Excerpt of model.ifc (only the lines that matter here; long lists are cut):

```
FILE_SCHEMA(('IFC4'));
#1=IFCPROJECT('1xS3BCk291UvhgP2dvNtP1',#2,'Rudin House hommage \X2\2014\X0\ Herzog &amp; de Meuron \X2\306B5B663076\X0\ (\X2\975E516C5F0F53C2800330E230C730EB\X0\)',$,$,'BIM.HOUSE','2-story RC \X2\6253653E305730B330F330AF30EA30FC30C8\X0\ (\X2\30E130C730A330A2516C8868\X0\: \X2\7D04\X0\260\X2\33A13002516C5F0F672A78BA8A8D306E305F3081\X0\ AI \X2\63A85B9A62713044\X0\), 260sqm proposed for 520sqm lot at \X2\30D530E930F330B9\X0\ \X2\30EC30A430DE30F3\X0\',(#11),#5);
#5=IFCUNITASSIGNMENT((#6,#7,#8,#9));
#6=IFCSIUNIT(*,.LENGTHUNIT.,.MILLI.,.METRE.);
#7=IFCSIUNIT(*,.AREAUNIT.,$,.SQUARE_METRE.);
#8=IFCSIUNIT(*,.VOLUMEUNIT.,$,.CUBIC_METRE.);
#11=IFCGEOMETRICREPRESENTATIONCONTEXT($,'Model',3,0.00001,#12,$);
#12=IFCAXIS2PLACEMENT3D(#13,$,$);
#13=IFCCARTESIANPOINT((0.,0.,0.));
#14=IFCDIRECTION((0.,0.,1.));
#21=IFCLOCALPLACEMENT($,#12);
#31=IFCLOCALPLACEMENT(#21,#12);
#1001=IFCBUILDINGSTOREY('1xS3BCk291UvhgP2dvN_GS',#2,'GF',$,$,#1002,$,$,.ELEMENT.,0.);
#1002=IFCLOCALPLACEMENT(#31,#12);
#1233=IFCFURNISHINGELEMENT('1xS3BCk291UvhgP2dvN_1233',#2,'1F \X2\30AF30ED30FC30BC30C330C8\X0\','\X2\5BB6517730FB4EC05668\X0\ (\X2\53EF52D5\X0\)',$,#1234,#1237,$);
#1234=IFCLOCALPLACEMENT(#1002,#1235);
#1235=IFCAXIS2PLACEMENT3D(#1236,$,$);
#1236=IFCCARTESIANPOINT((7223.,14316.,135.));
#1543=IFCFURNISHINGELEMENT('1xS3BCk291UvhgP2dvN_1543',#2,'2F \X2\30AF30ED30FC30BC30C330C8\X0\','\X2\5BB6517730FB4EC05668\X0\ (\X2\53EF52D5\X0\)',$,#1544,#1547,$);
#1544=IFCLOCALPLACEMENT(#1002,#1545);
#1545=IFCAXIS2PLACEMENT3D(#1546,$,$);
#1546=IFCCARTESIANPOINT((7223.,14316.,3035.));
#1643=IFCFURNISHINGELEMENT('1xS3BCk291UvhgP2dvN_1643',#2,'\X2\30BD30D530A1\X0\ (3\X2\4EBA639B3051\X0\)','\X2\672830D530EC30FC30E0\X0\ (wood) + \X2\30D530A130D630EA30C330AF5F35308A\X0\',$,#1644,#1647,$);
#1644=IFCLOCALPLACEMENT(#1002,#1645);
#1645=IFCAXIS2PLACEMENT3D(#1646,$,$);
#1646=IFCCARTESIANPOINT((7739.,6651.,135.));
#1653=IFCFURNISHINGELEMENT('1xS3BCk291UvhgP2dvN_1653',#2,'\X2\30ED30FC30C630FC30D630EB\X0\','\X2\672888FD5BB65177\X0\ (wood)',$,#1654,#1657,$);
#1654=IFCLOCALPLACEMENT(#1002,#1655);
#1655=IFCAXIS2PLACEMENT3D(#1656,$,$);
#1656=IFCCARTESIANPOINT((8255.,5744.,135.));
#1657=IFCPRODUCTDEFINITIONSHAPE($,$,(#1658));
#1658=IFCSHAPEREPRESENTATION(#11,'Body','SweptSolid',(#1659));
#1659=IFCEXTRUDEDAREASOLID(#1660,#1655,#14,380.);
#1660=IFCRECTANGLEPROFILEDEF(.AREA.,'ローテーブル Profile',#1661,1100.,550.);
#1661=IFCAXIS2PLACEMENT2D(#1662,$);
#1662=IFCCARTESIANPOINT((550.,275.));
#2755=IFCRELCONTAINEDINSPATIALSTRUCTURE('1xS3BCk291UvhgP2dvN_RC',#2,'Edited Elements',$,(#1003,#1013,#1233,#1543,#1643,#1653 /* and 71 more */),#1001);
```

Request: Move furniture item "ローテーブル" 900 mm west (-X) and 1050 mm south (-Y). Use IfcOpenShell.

```python
import ifcopenshell
import ifcopenshell.api.geometry
import ifcopenshell.util.placement
import ifcopenshell.util.unit

model = ifcopenshell.open("model.ifc")
unit_scale = ifcopenshell.util.unit.calculate_unit_scale(model)

item = model.by_guid("1xS3BCk291UvhgP2dvN_1653")
matrix = ifcopenshell.util.placement.get_local_placement(item.ObjectPlacement)
matrix[0, 3] -= 0.9 / unit_scale
matrix[1, 3] -= 1.05 / unit_scale
ifcopenshell.api.geometry.edit_object_placement(model, product=item, matrix=matrix, is_si=False)

print(ifcopenshell.util.placement.get_local_placement(item.ObjectPlacement).round(3) + 0.0)

model.write("model_rev.ifc")
```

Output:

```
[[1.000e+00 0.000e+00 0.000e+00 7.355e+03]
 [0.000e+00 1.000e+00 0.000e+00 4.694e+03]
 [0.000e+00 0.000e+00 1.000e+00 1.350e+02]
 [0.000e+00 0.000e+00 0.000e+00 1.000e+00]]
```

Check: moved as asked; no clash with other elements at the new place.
